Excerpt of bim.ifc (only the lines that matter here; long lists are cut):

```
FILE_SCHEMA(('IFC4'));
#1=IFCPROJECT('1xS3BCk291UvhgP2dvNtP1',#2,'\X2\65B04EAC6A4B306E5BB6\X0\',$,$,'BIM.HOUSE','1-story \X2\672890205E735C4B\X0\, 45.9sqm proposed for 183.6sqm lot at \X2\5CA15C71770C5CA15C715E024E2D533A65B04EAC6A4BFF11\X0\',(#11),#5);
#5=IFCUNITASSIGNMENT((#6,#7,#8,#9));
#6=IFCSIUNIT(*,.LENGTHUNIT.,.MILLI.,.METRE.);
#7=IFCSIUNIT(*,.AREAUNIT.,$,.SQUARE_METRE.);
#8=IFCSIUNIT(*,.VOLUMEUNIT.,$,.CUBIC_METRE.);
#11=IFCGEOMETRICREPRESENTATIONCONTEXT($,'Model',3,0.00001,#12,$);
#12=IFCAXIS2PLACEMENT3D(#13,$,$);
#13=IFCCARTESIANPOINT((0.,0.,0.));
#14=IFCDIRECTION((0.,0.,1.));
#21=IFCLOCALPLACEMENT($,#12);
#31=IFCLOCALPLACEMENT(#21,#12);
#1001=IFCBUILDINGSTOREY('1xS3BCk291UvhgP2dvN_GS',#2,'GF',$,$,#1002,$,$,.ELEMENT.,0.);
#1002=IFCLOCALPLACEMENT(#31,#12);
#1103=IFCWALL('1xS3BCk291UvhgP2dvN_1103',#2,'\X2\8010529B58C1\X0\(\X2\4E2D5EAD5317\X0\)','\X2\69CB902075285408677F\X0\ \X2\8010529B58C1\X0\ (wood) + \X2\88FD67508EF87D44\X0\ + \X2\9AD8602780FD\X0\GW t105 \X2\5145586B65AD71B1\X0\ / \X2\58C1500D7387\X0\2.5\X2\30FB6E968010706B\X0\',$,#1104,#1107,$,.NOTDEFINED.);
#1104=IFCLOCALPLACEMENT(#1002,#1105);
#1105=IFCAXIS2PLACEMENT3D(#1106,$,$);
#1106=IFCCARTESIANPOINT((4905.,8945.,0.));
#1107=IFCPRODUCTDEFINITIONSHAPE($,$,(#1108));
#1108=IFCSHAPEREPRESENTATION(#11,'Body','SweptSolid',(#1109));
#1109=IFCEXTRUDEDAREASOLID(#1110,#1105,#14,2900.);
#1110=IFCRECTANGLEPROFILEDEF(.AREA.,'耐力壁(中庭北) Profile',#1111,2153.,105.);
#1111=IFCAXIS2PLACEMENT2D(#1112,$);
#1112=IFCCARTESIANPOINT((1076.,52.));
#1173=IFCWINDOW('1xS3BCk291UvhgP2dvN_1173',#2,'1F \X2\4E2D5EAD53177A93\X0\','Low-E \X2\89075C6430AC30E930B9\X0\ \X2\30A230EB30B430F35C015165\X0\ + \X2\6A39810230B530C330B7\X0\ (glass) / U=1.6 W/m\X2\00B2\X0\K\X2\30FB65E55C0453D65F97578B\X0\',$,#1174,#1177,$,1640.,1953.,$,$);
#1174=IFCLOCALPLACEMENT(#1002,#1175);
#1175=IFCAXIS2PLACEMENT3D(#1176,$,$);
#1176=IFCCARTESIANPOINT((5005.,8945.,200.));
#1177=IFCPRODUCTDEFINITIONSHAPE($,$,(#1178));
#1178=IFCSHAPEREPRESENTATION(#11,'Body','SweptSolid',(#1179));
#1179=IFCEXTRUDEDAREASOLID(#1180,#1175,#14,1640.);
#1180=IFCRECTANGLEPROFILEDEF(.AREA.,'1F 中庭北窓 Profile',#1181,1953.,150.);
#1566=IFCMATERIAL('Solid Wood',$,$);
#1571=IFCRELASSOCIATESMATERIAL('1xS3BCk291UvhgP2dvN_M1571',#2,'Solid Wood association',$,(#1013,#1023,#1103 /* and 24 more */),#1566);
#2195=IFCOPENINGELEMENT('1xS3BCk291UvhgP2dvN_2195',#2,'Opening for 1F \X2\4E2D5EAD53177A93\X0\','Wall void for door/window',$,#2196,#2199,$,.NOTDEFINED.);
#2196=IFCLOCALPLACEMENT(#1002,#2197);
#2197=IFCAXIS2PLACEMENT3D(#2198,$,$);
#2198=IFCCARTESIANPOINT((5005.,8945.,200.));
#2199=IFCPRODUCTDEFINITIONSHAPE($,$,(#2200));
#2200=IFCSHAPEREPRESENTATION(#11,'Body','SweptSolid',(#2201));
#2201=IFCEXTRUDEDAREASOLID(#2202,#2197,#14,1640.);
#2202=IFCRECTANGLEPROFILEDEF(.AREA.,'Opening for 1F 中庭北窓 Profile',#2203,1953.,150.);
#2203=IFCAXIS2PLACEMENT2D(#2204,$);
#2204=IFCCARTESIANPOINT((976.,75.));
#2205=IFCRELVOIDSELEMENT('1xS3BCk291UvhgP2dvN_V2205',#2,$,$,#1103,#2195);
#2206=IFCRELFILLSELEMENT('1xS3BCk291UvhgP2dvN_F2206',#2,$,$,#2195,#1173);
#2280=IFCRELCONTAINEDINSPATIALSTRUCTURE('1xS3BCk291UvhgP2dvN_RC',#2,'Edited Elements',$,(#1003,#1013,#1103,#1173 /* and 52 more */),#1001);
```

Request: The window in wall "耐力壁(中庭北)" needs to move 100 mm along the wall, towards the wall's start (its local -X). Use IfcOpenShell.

```python
import ifcopenshell
import ifcopenshell.api.geometry
import ifcopenshell.util.placement
import ifcopenshell.util.unit

model = ifcopenshell.open("bim.ifc")
unit_scale = ifcopenshell.util.unit.calculate_unit_scale(model)

window = model.by_guid("1xS3BCk291UvhgP2dvN_1173")
opening = window.FillsVoids[0].RelatingOpeningElement
wall = opening.VoidsElements[0].RelatingBuildingElement

wall_matrix = ifcopenshell.util.placement.get_local_placement(wall.ObjectPlacement)
shift = wall_matrix[:3, 0] * -0.1 / unit_scale
before = ifcopenshell.util.placement.get_local_placement(window.ObjectPlacement)[:3, 3].copy()

# The window is not placed relative to its opening, so move both.
for product in (opening, window):
    matrix = ifcopenshell.util.placement.get_local_placement(product.ObjectPlacement)
    matrix[:3, 3] += shift
    ifcopenshell.api.geometry.edit_object_placement(model, product=product, matrix=matrix, is_si=False)

after = ifcopenshell.util.placement.get_local_placement(window.ObjectPlacement)[:3, 3]
print("window moved by", (after - before).round(3) + 0.0)

model.write("bim_rev.ifc")
```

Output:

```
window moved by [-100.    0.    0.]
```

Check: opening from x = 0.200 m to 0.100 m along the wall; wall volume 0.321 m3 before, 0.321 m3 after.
